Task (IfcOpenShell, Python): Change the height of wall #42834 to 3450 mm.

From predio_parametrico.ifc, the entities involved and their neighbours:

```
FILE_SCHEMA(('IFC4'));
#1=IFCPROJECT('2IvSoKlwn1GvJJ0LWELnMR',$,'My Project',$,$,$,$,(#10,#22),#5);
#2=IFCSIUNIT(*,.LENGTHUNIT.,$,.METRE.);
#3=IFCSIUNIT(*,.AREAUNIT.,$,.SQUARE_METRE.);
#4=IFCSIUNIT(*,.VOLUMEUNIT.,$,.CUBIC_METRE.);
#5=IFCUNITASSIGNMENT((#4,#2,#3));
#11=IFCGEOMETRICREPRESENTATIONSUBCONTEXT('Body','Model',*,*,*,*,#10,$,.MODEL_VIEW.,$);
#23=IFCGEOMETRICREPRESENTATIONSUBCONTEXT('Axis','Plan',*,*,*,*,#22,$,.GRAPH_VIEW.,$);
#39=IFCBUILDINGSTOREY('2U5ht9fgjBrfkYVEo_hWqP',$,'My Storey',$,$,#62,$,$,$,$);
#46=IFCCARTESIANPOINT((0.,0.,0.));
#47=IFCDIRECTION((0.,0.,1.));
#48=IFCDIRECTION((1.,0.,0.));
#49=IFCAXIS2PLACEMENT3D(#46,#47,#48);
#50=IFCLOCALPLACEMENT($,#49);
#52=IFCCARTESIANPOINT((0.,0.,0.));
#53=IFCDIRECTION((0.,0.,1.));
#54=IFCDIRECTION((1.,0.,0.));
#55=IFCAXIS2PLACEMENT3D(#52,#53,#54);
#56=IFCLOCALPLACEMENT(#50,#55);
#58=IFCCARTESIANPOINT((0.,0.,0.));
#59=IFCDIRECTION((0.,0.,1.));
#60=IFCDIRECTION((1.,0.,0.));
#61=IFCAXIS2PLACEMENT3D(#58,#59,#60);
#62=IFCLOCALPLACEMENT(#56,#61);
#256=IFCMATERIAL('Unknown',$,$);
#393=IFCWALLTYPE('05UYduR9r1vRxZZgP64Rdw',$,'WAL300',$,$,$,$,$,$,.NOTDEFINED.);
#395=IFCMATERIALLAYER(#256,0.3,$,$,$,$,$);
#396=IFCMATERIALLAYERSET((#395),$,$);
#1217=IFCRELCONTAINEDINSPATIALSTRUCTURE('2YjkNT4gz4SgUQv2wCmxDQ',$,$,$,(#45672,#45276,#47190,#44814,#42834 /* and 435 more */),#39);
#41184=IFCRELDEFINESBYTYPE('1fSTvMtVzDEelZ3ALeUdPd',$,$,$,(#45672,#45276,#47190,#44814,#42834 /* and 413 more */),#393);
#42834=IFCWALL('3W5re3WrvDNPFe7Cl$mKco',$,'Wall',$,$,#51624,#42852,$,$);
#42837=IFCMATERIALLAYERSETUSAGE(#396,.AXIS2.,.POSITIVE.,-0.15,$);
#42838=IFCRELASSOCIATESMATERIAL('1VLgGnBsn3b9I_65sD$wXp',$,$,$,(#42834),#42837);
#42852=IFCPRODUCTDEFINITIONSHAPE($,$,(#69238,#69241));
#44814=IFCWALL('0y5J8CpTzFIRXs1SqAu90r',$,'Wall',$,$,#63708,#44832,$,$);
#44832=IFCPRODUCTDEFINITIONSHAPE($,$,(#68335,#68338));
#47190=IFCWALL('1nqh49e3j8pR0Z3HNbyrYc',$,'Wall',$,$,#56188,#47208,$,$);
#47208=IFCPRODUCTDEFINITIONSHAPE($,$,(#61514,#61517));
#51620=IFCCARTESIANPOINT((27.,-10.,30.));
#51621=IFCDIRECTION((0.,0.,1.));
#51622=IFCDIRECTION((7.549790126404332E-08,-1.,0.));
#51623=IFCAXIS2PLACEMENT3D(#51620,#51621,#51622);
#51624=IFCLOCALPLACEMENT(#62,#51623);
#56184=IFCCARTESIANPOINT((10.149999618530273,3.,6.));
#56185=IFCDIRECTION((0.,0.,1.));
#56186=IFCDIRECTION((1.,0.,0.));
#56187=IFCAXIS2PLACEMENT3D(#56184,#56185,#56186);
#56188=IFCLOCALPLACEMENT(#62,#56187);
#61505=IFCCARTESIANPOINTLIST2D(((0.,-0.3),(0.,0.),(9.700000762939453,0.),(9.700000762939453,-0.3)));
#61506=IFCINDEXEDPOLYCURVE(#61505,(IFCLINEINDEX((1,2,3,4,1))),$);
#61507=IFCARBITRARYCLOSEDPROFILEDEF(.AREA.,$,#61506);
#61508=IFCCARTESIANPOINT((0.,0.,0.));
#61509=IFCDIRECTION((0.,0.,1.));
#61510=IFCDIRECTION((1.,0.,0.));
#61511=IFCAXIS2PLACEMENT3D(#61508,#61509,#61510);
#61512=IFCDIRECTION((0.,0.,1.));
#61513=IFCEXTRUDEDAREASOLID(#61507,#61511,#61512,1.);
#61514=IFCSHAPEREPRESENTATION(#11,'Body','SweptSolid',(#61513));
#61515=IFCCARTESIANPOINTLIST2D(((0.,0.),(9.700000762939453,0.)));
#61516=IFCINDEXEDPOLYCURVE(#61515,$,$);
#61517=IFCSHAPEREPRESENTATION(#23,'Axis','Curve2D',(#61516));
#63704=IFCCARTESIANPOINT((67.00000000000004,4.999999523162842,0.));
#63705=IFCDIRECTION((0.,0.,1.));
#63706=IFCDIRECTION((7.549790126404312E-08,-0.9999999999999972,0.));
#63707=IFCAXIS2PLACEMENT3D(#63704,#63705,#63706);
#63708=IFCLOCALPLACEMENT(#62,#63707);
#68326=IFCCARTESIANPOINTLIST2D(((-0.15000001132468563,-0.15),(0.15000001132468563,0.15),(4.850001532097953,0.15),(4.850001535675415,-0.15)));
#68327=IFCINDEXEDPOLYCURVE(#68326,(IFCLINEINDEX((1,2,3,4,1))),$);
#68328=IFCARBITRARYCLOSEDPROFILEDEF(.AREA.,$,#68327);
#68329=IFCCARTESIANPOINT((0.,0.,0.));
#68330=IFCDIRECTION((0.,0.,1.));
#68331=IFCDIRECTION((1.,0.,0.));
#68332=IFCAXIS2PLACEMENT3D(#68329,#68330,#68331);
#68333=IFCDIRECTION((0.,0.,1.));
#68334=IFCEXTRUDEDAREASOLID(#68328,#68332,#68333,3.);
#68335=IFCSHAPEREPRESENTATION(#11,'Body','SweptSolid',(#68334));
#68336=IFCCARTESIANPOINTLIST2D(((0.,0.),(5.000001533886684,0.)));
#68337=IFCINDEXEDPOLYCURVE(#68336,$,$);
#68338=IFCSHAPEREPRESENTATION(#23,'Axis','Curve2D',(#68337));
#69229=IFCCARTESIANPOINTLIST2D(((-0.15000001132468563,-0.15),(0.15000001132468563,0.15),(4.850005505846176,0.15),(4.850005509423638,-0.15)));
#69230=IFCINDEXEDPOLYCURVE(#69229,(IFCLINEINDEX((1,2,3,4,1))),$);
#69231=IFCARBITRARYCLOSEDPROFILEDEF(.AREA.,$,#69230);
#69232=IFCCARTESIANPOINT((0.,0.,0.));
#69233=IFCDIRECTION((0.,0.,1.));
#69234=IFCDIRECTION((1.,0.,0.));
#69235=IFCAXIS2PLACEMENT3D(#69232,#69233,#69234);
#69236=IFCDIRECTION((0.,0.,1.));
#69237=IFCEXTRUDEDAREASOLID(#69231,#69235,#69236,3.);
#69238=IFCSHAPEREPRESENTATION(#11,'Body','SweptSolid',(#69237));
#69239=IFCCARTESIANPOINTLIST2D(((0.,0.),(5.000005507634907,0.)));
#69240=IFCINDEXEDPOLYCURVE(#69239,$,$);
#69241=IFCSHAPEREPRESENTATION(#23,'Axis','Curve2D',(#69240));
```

```python
import ifcopenshell
import ifcopenshell.geom
import ifcopenshell.util.representation
import ifcopenshell.util.shape

model = ifcopenshell.open("predio_parametrico.ifc")
settings = ifcopenshell.geom.settings()


def volume(element):
    """Net volume in cubic metres, openings subtracted."""
    shape = ifcopenshell.geom.create_shape(settings, element)
    return ifcopenshell.util.shape.get_volume(shape.geometry)


wall = model.by_guid("3W5re3WrvDNPFe7Cl$mKco")
before = volume(wall)

body = ifcopenshell.util.representation.get_representation(wall, "Model", "Body")
solid = body.Items[0]
old_height = solid.Depth
solid.Depth = 3.45
after = volume(wall)

print(f"height {old_height:g} -> {solid.Depth:g}, volume {before:.3f} -> {after:.3f} m3")

model.write("predio_parametrico_edited.ifc")
```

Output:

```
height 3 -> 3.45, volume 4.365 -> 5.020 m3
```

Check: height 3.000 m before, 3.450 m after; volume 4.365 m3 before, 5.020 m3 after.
